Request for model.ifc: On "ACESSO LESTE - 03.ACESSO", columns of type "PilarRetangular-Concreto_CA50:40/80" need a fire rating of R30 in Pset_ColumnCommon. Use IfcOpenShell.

First a look at what the model holds.

```python
import ifcopenshell
import ifcopenshell.util.element

model = ifcopenshell.open("model.ifc")
print(model.schema)
storey = next(s for s in model.by_type("IfcBuildingStorey") if s.Name == "ACESSO LESTE - 03.ACESSO")
columns = [e for e in ifcopenshell.util.element.get_decomposition(storey) if e.is_a("IfcColumn")]
seen = {}
for e in columns:
    element_type = ifcopenshell.util.element.get_type(e)
    key = (element_type.Name if element_type != e and element_type else None, ifcopenshell.util.element.get_pset(e, "Pset_ColumnCommon", "FireRating"))
    seen[key] = seen.get(key, 0) + 1
for (name, value), count in sorted(seen.items(), key=str):
    print(count, "x", name, "|", value)
```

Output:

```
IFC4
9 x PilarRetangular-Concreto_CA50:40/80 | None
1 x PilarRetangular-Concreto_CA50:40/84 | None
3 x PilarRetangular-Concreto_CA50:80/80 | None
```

```python
import ifcopenshell
import ifcopenshell.api.pset
import ifcopenshell.util.element

model = ifcopenshell.open("model.ifc")

storey = next(s for s in model.by_type("IfcBuildingStorey") if s.Name == "ACESSO LESTE - 03.ACESSO")
columns = [e for e in ifcopenshell.util.element.get_decomposition(storey) if e.is_a("IfcColumn")]

count = 0
for e in columns:
    element_type = ifcopenshell.util.element.get_type(e)
    if element_type in (None, e) or element_type.Name != "PilarRetangular-Concreto_CA50:40/80":
        continue
    # add_pset returns the element's existing set when there is one.
    pset = ifcopenshell.api.pset.add_pset(model, product=e, name="Pset_ColumnCommon")
    ifcopenshell.api.pset.edit_pset(model, pset=pset, properties={"FireRating": "R30"})
    count += 1

print(count, "columns updated")

model.write("model_v2.ifc")
```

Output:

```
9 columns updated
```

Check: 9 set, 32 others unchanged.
